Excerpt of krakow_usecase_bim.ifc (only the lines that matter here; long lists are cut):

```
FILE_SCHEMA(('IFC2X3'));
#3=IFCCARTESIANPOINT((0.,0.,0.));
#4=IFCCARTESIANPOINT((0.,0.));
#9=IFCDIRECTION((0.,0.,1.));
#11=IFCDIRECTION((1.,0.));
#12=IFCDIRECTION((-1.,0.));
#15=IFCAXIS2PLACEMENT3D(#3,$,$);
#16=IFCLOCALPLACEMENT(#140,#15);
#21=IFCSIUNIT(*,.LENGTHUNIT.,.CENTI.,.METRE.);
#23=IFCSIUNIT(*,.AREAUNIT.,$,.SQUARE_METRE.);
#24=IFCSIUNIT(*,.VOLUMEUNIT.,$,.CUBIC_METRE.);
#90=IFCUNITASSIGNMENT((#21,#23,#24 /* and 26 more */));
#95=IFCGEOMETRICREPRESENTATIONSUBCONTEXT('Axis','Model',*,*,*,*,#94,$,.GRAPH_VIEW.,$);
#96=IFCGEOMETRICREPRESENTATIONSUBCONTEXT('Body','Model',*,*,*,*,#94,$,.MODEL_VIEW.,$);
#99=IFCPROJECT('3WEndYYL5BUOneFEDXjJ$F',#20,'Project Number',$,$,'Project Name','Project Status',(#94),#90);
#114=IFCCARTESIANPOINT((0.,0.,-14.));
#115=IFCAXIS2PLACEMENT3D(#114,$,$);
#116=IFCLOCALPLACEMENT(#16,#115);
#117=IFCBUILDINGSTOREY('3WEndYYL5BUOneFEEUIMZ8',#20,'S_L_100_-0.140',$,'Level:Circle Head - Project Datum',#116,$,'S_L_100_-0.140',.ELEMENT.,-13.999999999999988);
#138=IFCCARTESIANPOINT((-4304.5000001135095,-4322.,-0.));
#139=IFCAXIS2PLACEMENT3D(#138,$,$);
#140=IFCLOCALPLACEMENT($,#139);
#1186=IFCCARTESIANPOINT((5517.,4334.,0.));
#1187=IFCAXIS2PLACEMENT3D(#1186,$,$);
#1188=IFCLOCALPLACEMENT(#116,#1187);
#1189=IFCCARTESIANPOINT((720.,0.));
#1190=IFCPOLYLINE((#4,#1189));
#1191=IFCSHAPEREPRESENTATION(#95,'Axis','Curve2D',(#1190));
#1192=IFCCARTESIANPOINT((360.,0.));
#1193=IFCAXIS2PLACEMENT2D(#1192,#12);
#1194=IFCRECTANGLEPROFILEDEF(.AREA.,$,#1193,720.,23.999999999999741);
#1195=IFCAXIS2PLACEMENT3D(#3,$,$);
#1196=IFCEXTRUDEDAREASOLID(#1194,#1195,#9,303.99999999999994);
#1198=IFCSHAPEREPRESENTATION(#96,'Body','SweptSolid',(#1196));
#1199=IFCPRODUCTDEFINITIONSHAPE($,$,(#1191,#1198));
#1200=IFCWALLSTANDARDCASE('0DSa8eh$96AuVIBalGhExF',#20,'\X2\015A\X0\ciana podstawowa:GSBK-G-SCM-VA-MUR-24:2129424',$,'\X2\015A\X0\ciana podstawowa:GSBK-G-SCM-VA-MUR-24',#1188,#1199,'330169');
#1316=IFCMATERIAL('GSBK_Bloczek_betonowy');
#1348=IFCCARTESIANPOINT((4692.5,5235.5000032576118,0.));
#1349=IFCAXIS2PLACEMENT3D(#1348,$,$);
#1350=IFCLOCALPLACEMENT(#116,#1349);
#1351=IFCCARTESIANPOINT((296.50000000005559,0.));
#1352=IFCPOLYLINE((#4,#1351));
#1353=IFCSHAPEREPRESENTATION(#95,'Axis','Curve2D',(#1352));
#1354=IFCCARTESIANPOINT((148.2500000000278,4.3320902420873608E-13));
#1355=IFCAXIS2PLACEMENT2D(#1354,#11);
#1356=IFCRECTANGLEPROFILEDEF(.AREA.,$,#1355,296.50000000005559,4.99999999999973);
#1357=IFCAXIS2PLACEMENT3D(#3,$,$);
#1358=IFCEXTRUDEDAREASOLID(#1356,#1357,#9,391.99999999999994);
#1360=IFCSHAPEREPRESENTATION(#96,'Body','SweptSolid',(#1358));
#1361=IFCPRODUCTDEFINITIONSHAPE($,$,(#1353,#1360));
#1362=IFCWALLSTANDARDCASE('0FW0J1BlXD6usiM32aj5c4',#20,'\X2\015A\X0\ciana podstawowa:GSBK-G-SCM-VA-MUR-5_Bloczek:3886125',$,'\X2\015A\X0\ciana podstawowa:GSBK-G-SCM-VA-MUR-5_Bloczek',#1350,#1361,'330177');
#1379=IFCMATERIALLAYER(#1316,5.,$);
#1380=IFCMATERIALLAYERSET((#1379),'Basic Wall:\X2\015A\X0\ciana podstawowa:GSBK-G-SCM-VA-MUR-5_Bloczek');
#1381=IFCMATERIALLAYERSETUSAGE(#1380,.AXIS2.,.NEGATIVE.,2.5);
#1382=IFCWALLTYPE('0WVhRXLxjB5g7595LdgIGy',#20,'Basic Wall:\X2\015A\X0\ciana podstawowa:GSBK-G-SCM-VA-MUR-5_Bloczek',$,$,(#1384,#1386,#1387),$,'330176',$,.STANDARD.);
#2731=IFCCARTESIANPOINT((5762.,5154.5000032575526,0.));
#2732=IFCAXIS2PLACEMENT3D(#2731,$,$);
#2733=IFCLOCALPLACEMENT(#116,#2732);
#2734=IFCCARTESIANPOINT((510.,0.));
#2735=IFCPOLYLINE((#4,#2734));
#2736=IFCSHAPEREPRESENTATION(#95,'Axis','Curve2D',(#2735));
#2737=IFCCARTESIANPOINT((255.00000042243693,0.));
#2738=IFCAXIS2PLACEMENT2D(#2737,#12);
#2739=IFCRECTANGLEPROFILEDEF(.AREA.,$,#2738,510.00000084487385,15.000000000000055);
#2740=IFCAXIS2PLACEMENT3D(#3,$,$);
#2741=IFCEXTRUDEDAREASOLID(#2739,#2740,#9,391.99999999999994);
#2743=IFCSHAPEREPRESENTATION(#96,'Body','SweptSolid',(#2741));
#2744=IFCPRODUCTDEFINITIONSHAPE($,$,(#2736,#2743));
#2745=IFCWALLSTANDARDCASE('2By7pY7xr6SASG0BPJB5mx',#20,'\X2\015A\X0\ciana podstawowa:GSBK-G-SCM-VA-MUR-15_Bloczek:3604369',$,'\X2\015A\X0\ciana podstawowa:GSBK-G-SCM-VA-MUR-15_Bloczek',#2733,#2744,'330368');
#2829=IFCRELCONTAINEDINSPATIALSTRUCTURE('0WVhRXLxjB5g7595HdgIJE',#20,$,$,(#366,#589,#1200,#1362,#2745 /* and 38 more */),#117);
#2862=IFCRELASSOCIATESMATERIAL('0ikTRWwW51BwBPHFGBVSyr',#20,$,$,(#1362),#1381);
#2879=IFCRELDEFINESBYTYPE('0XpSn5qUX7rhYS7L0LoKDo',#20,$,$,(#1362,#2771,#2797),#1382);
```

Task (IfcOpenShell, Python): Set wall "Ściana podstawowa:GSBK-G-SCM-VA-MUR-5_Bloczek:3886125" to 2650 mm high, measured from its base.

```python
import ifcopenshell
import ifcopenshell.geom
import ifcopenshell.util.representation
import ifcopenshell.util.shape
import ifcopenshell.util.unit

model = ifcopenshell.open("krakow_usecase_bim.ifc")
unit_scale = ifcopenshell.util.unit.calculate_unit_scale(model)
settings = ifcopenshell.geom.settings()


def volume(element):
    """Net volume in cubic metres, openings subtracted."""
    shape = ifcopenshell.geom.create_shape(settings, element)
    return ifcopenshell.util.shape.get_volume(shape.geometry)


wall = model.by_guid("0FW0J1BlXD6usiM32aj5c4")
before = volume(wall)

body = ifcopenshell.util.representation.get_representation(wall, "Model", "Body")
solid = body.Items[0]
old_height = solid.Depth
solid.Depth = 2.65 / unit_scale
after = volume(wall)

print(f"height {old_height:g} -> {solid.Depth:g}, volume {before:.3f} -> {after:.3f} m3")

model.write("krakow_usecase_bim-out.ifc")
```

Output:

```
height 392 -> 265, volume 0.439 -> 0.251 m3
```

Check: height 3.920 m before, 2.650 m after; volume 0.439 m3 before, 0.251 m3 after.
